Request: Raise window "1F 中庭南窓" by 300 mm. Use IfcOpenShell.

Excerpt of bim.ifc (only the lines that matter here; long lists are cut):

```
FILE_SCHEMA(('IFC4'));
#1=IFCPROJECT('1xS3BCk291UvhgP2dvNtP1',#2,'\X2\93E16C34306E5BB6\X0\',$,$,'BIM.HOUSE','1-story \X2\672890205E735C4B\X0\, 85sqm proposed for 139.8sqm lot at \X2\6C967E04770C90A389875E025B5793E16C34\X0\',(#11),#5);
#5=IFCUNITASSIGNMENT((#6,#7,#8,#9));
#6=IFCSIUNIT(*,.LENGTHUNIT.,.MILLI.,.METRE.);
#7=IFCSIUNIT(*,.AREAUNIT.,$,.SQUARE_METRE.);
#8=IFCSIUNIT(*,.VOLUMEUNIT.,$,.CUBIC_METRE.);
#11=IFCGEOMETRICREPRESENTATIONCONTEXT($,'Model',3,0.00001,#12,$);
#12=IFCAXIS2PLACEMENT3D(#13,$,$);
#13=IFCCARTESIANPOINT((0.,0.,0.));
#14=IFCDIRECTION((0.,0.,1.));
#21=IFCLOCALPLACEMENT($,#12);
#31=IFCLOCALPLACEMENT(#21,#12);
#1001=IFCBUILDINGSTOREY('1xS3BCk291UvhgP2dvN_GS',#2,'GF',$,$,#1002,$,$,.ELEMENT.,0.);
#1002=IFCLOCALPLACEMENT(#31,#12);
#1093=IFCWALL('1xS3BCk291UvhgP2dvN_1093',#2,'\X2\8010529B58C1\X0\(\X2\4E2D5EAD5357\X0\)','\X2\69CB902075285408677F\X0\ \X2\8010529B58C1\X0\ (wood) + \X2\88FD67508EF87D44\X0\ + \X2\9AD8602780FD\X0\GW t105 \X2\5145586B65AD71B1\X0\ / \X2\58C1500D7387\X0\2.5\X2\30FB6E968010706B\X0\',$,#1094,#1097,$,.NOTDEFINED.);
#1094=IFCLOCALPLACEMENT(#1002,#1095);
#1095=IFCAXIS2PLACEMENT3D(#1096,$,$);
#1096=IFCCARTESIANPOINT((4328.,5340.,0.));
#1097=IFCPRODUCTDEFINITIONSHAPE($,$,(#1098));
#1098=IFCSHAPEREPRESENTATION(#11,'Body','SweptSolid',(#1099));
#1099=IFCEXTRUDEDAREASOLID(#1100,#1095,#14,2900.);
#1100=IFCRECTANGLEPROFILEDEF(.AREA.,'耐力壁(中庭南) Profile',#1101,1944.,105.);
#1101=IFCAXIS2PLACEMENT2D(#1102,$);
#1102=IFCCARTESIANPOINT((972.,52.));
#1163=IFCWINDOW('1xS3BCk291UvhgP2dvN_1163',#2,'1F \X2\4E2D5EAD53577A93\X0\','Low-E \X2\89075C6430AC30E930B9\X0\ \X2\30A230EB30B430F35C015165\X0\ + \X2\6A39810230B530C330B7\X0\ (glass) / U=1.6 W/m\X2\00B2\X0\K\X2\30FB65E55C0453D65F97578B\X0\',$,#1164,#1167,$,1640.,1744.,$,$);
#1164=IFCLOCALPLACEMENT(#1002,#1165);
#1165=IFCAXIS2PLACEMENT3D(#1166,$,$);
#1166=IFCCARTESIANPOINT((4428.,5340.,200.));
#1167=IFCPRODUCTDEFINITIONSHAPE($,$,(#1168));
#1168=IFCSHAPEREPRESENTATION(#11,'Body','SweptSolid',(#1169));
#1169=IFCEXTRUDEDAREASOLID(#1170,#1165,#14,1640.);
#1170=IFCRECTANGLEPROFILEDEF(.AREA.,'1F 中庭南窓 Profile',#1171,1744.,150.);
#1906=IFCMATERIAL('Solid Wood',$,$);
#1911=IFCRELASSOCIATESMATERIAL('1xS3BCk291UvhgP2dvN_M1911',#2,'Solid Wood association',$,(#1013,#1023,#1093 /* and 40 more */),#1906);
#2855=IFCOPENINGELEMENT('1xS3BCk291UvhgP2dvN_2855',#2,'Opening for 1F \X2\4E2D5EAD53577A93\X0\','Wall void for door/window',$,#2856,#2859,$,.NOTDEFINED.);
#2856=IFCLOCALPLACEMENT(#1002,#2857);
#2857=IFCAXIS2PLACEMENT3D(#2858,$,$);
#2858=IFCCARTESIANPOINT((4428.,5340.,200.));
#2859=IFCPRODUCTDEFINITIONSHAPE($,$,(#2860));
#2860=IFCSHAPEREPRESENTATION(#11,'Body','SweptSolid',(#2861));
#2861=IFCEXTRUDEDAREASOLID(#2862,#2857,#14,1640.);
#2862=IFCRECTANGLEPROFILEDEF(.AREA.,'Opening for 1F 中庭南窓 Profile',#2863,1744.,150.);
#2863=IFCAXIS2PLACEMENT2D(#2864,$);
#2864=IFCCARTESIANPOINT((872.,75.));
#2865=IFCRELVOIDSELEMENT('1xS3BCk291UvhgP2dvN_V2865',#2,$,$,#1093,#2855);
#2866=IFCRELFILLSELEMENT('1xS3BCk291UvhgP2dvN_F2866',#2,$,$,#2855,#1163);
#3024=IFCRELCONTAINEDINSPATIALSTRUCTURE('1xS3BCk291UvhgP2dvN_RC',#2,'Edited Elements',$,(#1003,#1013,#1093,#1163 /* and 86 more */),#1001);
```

```python
import numpy as np
import ifcopenshell
import ifcopenshell.api.geometry
import ifcopenshell.util.placement
import ifcopenshell.util.unit

model = ifcopenshell.open("bim.ifc")
unit_scale = ifcopenshell.util.unit.calculate_unit_scale(model)

window = model.by_guid("1xS3BCk291UvhgP2dvN_1163")
opening = window.FillsVoids[0].RelatingOpeningElement
dz = 0.3 / unit_scale

shift = np.array([0.0, 0.0, dz])
# The window is not placed relative to its opening, so move both.
for product in (opening, window):
    matrix = ifcopenshell.util.placement.get_local_placement(product.ObjectPlacement)
    matrix[:3, 3] += shift
    ifcopenshell.api.geometry.edit_object_placement(model, product=product, matrix=matrix, is_si=False)

print(f"moved by {dz * unit_scale:+.3f} m")

model.write("bim_rev.ifc")
```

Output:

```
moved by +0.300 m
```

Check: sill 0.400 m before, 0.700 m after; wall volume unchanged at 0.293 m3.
